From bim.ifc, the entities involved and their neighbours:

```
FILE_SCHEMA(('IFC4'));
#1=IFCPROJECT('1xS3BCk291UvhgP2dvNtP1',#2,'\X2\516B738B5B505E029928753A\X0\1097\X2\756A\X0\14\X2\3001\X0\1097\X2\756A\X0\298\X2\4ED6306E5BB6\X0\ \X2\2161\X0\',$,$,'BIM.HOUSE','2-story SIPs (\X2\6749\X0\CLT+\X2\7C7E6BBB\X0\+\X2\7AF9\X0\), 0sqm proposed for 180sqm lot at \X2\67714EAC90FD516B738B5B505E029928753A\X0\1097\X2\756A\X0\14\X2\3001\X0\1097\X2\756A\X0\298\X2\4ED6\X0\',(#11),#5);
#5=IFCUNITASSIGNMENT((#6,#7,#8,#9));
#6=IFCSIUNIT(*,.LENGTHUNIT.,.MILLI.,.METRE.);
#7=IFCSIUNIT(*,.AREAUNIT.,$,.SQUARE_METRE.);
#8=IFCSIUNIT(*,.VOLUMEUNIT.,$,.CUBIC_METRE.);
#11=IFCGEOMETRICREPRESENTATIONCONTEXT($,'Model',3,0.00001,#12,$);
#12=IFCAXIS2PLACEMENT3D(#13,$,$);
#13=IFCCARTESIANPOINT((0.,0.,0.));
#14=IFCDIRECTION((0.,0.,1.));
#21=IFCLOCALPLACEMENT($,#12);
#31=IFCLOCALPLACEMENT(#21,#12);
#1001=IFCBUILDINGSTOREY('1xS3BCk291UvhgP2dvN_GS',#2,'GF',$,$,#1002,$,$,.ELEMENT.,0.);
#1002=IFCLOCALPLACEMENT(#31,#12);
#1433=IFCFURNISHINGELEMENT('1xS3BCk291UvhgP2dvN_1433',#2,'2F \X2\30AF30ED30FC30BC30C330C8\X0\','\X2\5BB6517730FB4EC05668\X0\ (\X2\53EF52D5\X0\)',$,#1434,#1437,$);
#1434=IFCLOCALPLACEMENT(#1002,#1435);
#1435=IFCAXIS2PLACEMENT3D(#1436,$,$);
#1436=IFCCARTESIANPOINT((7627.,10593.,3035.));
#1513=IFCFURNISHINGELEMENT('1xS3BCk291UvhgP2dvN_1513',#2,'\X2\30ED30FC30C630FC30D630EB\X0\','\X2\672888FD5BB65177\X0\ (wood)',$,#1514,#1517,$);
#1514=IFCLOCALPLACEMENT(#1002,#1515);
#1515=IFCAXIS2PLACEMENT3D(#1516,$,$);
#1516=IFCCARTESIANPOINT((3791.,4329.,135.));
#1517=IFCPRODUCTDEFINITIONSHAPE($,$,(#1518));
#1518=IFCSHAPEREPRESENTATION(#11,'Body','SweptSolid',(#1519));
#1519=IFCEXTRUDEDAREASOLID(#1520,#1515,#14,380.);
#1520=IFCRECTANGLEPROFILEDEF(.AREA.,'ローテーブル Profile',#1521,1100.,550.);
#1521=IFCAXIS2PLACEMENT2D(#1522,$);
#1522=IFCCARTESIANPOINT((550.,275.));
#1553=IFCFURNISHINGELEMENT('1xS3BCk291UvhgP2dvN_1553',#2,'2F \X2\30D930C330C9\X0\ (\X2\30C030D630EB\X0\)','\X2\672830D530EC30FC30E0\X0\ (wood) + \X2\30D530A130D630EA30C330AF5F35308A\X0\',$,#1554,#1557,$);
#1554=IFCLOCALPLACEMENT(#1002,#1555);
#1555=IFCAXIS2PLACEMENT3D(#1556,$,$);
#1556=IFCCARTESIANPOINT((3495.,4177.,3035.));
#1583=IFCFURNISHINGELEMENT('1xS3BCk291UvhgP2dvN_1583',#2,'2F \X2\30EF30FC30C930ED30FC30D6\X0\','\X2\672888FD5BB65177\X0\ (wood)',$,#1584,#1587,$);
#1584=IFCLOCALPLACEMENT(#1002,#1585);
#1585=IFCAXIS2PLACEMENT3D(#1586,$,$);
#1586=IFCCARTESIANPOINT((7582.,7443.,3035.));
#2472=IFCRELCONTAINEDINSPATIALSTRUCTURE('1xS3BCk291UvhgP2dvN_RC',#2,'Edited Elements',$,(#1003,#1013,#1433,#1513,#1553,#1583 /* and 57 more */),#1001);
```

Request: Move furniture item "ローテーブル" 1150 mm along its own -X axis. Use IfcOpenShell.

```python
import ifcopenshell
import ifcopenshell.api.geometry
import ifcopenshell.util.placement
import ifcopenshell.util.unit

model = ifcopenshell.open("bim.ifc")
unit_scale = ifcopenshell.util.unit.calculate_unit_scale(model)

item = model.by_guid("1xS3BCk291UvhgP2dvN_1513")
matrix = ifcopenshell.util.placement.get_local_placement(item.ObjectPlacement)
matrix[:3, 3] -= matrix[:3, 0] * 1.15 / unit_scale
ifcopenshell.api.geometry.edit_object_placement(model, product=item, matrix=matrix, is_si=False)

print(ifcopenshell.util.placement.get_local_placement(item.ObjectPlacement).round(3) + 0.0)

model.write("bim_edited.ifc")
```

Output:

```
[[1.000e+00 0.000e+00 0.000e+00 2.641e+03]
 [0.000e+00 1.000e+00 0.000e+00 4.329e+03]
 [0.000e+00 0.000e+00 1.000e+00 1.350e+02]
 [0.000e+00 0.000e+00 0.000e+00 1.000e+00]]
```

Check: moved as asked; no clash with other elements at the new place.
